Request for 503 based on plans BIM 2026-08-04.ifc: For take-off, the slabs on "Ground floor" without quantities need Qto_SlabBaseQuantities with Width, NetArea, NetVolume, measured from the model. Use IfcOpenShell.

First a look at what the model holds.

```python
import ifcopenshell
import ifcopenshell.util.element
import ifcopenshell.util.unit

model = ifcopenshell.open("503 based on plans BIM 2026-08-04.ifc")
print(model.schema)
for unit_type in ("LENGTHUNIT", "AREAUNIT", "VOLUMEUNIT"):
    print(unit_type, ifcopenshell.util.unit.calculate_unit_scale(model, unit_type))
storey = next(s for s in model.by_type("IfcBuildingStorey") if s.Name == "Ground floor")
slabs = [e for e in ifcopenshell.util.element.get_decomposition(storey) if e.is_a("IfcSlab")]
for e in sorted(slabs, key=lambda e: e.id()):
    print(e.id(), e.is_a(), e.Name, list(ifcopenshell.util.element.get_psets(e, qtos_only=True)), sep=" | ")
```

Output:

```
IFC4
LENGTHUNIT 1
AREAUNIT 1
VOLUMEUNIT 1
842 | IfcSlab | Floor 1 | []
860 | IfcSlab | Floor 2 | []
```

```python
import ifcopenshell
import ifcopenshell.api.pset
import ifcopenshell.geom
import ifcopenshell.util.element
import ifcopenshell.util.shape
import ifcopenshell.util.unit

model = ifcopenshell.open("503 based on plans BIM 2026-08-04.ifc")
unit_scale = ifcopenshell.util.unit.calculate_unit_scale(model)
area_scale = ifcopenshell.util.unit.calculate_unit_scale(model, "AREAUNIT")
volume_scale = ifcopenshell.util.unit.calculate_unit_scale(model, "VOLUMEUNIT")
settings = ifcopenshell.geom.settings()

storey = next(s for s in model.by_type("IfcBuildingStorey") if s.Name == "Ground floor")
slabs = [e for e in ifcopenshell.util.element.get_decomposition(storey) if e.is_a("IfcSlab")]

for e in sorted(slabs, key=lambda e: e.id()):
    if ifcopenshell.util.element.get_psets(e, qtos_only=True, should_inherit=False):
        continue
    # Geometry comes back in metres, in the element's own axes.
    shape = ifcopenshell.geom.create_shape(settings, e)
    values = {
        "Width": ifcopenshell.util.shape.get_z(shape.geometry) / unit_scale,
        "NetArea": ifcopenshell.util.shape.get_footprint_area(shape.geometry) / area_scale,
        "NetVolume": ifcopenshell.util.shape.get_volume(shape.geometry) / volume_scale,
    }
    qto = ifcopenshell.api.pset.add_qto(model, product=e, name="Qto_SlabBaseQuantities")
    ifcopenshell.api.pset.edit_qto(model, qto=qto, properties=values)
    print(e.id(), {k: round(v, 3) for k, v in values.items()})

model.write("503 based on plans BIM 2026-08-04_rev.ifc")
```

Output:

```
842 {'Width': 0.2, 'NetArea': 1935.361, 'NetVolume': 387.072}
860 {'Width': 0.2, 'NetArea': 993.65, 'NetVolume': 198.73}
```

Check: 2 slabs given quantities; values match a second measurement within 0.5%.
